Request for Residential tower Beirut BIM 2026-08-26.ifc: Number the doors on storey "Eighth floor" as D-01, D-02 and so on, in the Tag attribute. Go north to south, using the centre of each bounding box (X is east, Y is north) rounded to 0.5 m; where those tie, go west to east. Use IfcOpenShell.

First a look at what the model holds.

```python
import ifcopenshell
import ifcopenshell.util.element
import ifcopenshell.util.placement

model = ifcopenshell.open("Residential tower Beirut BIM 2026-08-26.ifc")
print(model.schema)
storey = next(s for s in model.by_type("IfcBuildingStorey") if s.Name == "Eighth floor")
doors = [e for e in ifcopenshell.util.element.get_decomposition(storey) if e.is_a("IfcDoor")]
for e in sorted(doors, key=lambda e: e.id()):
    origin = ifcopenshell.util.placement.get_local_placement(e.ObjectPlacement)[:3, 3]
    print(e.id(), e.Tag, e.Name, origin.round(2) + 0.0, sep=" | ")
```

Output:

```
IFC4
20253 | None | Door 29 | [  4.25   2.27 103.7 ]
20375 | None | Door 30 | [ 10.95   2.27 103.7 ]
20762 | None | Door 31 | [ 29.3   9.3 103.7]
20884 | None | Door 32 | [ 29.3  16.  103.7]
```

```python
import ifcopenshell
import ifcopenshell.geom
import ifcopenshell.util.element
import ifcopenshell.util.shape

model = ifcopenshell.open("Residential tower Beirut BIM 2026-08-26.ifc")
settings = ifcopenshell.geom.settings()
settings.set("use-world-coords", True)


def centre(element):
    shape = ifcopenshell.geom.create_shape(settings, element)
    return ifcopenshell.util.shape.get_bbox_centroid(shape.geometry)


storey = next(s for s in model.by_type("IfcBuildingStorey") if s.Name == "Eighth floor")
doors = [e for e in ifcopenshell.util.element.get_decomposition(storey) if e.is_a("IfcDoor")]

# Insertion points can sit at a corner or the storey origin, so sort by the geometry (in metres).
centres = {e: centre(e) for e in doors}
doors.sort(key=lambda e: (-round(centres[e][1] / 0.5), centres[e][0]))

for i, e in enumerate(doors, start=1):
    number = f"D-{i:02d}"
    e.Tag = number
    print(e.id(), number)

model.write("Residential tower Beirut BIM 2026-08-26_rev.ifc")
```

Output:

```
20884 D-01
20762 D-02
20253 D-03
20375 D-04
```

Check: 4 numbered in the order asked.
